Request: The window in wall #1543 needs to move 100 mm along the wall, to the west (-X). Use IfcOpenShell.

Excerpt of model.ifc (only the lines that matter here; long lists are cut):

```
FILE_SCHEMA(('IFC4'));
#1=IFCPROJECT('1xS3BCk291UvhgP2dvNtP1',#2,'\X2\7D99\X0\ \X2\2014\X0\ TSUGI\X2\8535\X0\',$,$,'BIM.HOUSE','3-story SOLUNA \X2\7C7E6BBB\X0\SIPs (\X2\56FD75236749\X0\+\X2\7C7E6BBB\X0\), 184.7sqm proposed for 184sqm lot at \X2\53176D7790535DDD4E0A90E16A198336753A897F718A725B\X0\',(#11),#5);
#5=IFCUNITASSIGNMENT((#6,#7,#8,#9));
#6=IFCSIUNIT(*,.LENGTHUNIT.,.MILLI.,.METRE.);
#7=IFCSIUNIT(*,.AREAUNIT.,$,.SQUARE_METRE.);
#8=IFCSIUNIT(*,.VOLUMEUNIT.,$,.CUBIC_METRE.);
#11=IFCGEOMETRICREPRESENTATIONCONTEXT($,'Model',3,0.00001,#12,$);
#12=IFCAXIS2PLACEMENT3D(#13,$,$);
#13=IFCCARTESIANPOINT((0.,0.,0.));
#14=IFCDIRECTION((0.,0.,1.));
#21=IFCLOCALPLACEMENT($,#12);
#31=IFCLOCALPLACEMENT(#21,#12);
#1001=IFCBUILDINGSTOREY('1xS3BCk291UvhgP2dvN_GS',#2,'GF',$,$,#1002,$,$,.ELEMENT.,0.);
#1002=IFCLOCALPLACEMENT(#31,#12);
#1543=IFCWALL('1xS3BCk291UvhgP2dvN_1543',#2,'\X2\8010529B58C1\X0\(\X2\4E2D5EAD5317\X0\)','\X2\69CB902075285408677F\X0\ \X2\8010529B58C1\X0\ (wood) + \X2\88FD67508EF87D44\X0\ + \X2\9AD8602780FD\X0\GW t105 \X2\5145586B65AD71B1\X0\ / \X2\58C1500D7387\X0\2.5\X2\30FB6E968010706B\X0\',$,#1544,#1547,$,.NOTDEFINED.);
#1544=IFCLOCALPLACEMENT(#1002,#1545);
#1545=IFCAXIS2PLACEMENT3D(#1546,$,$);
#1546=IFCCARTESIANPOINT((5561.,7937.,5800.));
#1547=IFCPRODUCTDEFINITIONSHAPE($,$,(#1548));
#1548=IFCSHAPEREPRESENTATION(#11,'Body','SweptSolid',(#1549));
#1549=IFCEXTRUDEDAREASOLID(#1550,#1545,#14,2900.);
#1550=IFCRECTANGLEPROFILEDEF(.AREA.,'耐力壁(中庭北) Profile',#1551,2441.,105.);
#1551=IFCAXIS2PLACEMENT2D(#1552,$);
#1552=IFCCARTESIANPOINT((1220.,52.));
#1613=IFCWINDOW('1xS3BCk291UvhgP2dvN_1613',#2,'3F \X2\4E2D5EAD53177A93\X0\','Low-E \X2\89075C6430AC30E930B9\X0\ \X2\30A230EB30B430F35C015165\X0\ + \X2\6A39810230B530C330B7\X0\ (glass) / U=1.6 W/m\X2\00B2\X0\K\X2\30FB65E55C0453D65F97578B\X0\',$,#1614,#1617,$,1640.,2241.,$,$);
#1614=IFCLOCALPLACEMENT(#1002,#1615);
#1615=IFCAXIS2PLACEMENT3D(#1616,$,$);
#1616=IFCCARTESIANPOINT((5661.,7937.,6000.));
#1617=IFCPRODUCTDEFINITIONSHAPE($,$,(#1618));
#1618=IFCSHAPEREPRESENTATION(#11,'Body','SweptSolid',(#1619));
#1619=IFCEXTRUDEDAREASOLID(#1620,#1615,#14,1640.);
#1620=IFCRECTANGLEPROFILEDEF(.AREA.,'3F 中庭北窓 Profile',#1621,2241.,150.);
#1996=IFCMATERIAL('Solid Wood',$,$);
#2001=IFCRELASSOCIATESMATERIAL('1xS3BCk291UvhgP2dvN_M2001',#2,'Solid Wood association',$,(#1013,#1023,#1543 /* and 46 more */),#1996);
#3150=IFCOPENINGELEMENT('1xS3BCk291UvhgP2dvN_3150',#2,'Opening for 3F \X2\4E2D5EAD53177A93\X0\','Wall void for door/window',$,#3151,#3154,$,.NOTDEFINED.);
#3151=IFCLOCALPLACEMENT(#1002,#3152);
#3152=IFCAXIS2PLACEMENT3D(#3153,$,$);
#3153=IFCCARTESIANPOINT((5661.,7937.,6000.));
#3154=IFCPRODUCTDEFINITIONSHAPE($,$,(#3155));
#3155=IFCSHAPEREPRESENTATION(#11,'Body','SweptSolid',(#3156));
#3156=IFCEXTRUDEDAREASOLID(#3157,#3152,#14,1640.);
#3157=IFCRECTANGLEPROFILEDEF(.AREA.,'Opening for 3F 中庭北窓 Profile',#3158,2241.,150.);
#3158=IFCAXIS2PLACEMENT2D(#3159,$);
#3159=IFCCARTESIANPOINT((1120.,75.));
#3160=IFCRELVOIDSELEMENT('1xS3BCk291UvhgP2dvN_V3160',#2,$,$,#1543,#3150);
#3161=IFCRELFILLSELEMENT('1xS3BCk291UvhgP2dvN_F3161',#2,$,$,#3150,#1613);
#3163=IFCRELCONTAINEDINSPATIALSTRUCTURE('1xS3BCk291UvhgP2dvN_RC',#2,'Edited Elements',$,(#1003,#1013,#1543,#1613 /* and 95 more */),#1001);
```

```python
import ifcopenshell
import ifcopenshell.api.geometry
import ifcopenshell.util.placement
import ifcopenshell.util.unit

model = ifcopenshell.open("model.ifc")
unit_scale = ifcopenshell.util.unit.calculate_unit_scale(model)

window = model.by_guid("1xS3BCk291UvhgP2dvN_1613")
opening = window.FillsVoids[0].RelatingOpeningElement
wall = opening.VoidsElements[0].RelatingBuildingElement

wall_matrix = ifcopenshell.util.placement.get_local_placement(wall.ObjectPlacement)
shift = wall_matrix[:3, 0] * -0.1 / unit_scale
before = ifcopenshell.util.placement.get_local_placement(window.ObjectPlacement)[:3, 3].copy()

# The window is not placed relative to its opening, so move both.
for product in (opening, window):
    matrix = ifcopenshell.util.placement.get_local_placement(product.ObjectPlacement)
    matrix[:3, 3] += shift
    ifcopenshell.api.geometry.edit_object_placement(model, product=product, matrix=matrix, is_si=False)

after = ifcopenshell.util.placement.get_local_placement(window.ObjectPlacement)[:3, 3]
print("window moved by", (after - before).round(3) + 0.0)

model.write("model_edited.ifc")
```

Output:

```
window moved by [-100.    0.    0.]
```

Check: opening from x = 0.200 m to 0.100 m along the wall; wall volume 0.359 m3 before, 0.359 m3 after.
